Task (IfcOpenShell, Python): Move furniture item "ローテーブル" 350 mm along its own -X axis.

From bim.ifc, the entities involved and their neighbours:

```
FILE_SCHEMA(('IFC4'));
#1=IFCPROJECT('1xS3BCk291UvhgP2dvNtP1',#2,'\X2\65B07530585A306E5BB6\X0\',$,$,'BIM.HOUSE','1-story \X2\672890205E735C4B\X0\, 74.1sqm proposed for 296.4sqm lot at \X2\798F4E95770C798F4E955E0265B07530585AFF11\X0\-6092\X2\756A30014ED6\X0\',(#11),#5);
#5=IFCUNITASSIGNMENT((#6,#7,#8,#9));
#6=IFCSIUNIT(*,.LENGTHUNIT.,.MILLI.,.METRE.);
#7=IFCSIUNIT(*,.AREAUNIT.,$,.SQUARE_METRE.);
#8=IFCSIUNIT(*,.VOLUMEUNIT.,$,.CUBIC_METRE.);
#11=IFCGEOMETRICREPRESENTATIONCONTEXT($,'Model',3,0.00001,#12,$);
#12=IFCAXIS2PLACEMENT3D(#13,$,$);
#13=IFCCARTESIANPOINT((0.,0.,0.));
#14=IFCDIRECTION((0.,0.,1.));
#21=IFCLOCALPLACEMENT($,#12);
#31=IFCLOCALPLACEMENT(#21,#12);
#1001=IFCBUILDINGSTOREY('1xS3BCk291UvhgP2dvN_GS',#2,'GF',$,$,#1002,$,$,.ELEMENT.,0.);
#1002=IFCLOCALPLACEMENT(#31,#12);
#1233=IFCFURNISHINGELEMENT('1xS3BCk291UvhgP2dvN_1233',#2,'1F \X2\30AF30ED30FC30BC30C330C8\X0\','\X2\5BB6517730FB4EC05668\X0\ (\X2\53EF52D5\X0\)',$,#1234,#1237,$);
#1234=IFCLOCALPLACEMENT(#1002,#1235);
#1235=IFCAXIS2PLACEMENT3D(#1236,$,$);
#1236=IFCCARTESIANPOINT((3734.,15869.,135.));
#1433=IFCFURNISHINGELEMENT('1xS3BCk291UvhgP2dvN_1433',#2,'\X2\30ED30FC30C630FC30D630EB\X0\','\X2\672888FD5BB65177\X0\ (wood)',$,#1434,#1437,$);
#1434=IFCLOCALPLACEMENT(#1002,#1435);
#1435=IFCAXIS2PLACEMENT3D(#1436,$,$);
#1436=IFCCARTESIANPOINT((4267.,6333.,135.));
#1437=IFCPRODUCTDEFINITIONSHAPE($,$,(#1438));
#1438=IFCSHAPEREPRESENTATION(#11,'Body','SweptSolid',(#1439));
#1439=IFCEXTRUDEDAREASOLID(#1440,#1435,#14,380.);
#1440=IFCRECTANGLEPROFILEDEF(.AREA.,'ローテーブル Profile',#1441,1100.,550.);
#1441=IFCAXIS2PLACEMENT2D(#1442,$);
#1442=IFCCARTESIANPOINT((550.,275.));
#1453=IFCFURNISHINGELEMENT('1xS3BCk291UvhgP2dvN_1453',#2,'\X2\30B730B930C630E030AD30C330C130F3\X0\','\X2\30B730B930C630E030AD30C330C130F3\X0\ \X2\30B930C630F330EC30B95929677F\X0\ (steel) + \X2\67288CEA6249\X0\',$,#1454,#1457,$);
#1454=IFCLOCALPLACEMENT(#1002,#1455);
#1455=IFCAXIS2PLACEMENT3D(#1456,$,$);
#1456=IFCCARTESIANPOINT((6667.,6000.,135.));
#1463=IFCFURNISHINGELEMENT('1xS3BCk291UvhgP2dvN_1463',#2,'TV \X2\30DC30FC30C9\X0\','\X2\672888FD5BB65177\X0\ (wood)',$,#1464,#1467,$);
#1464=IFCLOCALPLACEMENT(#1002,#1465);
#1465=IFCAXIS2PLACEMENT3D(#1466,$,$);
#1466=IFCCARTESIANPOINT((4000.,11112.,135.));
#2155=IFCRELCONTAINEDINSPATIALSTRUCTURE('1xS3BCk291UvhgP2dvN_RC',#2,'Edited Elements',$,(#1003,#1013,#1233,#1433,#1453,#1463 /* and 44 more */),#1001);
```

```python
import ifcopenshell
import ifcopenshell.api.geometry
import ifcopenshell.util.placement

model = ifcopenshell.open("bim.ifc")

item = model.by_id(1433)
matrix = ifcopenshell.util.placement.get_local_placement(item.ObjectPlacement)
matrix[:3, 3] -= matrix[:3, 0] * 350.0
ifcopenshell.api.geometry.edit_object_placement(model, product=item, matrix=matrix, is_si=False)

print(ifcopenshell.util.placement.get_local_placement(item.ObjectPlacement).round(3) + 0.0)

model.write("bim_rev.ifc")
```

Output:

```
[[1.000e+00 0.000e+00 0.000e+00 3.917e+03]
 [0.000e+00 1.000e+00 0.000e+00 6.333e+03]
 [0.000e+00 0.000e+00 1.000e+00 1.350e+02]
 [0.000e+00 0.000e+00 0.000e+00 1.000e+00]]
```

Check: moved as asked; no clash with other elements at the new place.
